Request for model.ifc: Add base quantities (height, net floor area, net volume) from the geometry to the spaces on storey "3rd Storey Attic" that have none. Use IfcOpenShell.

First a look at what the model holds.

```python
import ifcopenshell
import ifcopenshell.util.element
import ifcopenshell.util.unit

model = ifcopenshell.open("model.ifc")
print(model.schema)
for unit_type in ("LENGTHUNIT", "AREAUNIT", "VOLUMEUNIT"):
    print(unit_type, ifcopenshell.util.unit.calculate_unit_scale(model, unit_type))
storey = next(s for s in model.by_type("IfcBuildingStorey") if s.Name == "3rd Storey Attic")
spaces = [e for e in ifcopenshell.util.element.get_decomposition(storey) if e.is_a("IfcSpace")]
for e in sorted(spaces, key=lambda e: e.id()):
    print(e.id(), e.is_a(), e.Name, list(ifcopenshell.util.element.get_psets(e, qtos_only=True)), sep=" | ")
```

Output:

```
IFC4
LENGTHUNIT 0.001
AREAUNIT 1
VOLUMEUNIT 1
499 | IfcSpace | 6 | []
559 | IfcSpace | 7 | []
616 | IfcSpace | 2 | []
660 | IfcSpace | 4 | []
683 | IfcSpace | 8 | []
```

```python
import ifcopenshell
import ifcopenshell.api.pset
import ifcopenshell.geom
import ifcopenshell.util.element
import ifcopenshell.util.shape
import ifcopenshell.util.unit

model = ifcopenshell.open("model.ifc")
unit_scale = ifcopenshell.util.unit.calculate_unit_scale(model)
area_scale = ifcopenshell.util.unit.calculate_unit_scale(model, "AREAUNIT")
volume_scale = ifcopenshell.util.unit.calculate_unit_scale(model, "VOLUMEUNIT")
settings = ifcopenshell.geom.settings()

storey = next(s for s in model.by_type("IfcBuildingStorey") if s.Name == "3rd Storey Attic")
spaces = [e for e in ifcopenshell.util.element.get_decomposition(storey) if e.is_a("IfcSpace")]

for e in sorted(spaces, key=lambda e: e.id()):
    if ifcopenshell.util.element.get_psets(e, qtos_only=True, should_inherit=False):
        continue
    # Geometry comes back in metres, in the element's own axes.
    shape = ifcopenshell.geom.create_shape(settings, e)
    values = {
        "Height": ifcopenshell.util.shape.get_z(shape.geometry) / unit_scale,
        "NetFloorArea": ifcopenshell.util.shape.get_footprint_area(shape.geometry) / area_scale,
        "NetVolume": ifcopenshell.util.shape.get_volume(shape.geometry) / volume_scale,
    }
    qto = ifcopenshell.api.pset.add_qto(model, product=e, name="Qto_SpaceBaseQuantities")
    ifcopenshell.api.pset.edit_qto(model, qto=qto, properties=values)
    print(e.id(), {k: round(v, 3) for k, v in values.items()})

model.write("model-out.ifc")
```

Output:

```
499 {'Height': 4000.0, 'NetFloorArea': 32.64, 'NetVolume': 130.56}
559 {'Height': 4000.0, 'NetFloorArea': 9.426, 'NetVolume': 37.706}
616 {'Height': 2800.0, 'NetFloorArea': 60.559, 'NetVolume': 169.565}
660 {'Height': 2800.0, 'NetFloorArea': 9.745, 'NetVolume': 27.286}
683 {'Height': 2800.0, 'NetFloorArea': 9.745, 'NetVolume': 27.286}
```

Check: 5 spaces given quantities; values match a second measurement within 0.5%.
